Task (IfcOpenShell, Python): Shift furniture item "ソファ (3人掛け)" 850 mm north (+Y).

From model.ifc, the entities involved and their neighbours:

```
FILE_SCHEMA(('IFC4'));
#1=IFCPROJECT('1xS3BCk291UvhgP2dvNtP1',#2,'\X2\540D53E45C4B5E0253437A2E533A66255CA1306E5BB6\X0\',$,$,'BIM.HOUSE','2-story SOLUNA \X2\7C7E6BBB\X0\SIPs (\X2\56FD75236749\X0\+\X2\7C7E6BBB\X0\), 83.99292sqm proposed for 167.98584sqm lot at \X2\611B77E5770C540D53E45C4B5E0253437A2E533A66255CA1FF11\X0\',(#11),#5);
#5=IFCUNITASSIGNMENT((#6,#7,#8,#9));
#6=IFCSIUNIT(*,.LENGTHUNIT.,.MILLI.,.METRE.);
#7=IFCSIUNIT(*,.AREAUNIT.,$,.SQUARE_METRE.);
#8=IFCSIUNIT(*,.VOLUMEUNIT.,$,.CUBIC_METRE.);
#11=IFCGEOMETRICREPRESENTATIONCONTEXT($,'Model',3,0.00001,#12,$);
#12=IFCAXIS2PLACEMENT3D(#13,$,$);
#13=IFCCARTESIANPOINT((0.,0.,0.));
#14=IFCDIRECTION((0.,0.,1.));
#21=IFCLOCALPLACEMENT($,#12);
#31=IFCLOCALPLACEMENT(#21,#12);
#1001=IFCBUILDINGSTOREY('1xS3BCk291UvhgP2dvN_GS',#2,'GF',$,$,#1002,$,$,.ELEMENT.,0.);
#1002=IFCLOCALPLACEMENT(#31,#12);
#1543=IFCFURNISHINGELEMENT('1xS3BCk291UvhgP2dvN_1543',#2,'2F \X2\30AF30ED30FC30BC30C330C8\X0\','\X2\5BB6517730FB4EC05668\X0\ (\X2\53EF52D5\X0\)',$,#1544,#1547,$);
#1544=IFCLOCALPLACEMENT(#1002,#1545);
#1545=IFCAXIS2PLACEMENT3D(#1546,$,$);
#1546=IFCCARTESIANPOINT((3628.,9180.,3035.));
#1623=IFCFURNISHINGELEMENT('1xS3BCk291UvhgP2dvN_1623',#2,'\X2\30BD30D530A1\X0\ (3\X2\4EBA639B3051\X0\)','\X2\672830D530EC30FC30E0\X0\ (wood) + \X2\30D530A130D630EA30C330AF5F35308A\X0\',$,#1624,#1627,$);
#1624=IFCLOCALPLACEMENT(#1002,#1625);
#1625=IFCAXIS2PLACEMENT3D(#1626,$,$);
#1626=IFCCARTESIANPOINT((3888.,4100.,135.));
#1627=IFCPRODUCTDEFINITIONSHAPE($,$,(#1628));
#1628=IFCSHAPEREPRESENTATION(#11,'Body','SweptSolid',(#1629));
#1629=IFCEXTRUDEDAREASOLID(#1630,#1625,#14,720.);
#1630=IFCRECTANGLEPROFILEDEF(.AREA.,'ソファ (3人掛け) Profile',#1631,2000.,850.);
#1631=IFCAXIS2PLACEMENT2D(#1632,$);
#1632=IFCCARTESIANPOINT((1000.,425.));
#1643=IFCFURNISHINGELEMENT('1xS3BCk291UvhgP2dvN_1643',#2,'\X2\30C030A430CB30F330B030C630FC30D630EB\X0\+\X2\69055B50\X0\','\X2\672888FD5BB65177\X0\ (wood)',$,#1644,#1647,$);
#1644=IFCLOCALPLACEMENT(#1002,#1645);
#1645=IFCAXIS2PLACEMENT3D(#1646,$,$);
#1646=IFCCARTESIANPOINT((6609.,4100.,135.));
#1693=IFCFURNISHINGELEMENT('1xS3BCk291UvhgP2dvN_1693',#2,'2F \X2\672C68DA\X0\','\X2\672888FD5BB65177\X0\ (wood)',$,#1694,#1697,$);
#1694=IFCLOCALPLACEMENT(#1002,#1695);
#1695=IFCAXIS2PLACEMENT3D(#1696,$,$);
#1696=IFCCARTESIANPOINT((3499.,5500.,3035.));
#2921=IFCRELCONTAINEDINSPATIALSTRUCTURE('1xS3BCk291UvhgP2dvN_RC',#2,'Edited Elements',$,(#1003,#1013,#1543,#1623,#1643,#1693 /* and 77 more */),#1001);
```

```python
import ifcopenshell
import ifcopenshell.api.geometry
import ifcopenshell.util.placement
import ifcopenshell.util.unit

model = ifcopenshell.open("model.ifc")
unit_scale = ifcopenshell.util.unit.calculate_unit_scale(model)

item = model.by_guid("1xS3BCk291UvhgP2dvN_1623")
matrix = ifcopenshell.util.placement.get_local_placement(item.ObjectPlacement)
matrix[1, 3] += 0.85 / unit_scale
ifcopenshell.api.geometry.edit_object_placement(model, product=item, matrix=matrix, is_si=False)

print(ifcopenshell.util.placement.get_local_placement(item.ObjectPlacement).round(3) + 0.0)

model.write("model_v2.ifc")
```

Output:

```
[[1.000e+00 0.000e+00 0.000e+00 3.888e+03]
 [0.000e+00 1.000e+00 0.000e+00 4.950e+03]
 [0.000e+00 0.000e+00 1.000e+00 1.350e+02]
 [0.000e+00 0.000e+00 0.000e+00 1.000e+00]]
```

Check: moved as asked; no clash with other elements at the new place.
